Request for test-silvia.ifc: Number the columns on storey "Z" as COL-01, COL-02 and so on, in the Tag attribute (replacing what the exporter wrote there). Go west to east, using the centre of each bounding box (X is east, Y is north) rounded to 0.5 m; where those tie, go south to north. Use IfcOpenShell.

First a look at what the model holds.

```python
import ifcopenshell
import ifcopenshell.util.element
import ifcopenshell.util.placement

model = ifcopenshell.open("test-silvia.ifc")
print(model.schema)
storey = next(s for s in model.by_type("IfcBuildingStorey") if s.Name == "Z")
columns = [e for e in ifcopenshell.util.element.get_decomposition(storey) if e.is_a("IfcColumn")]
for e in sorted(columns, key=lambda e: e.id()):
    origin = ifcopenshell.util.placement.get_local_placement(e.ObjectPlacement)[:3, 3]
    print(e.id(), e.Tag, e.Name, origin.round(2) + 0.0, sep=" | ")
```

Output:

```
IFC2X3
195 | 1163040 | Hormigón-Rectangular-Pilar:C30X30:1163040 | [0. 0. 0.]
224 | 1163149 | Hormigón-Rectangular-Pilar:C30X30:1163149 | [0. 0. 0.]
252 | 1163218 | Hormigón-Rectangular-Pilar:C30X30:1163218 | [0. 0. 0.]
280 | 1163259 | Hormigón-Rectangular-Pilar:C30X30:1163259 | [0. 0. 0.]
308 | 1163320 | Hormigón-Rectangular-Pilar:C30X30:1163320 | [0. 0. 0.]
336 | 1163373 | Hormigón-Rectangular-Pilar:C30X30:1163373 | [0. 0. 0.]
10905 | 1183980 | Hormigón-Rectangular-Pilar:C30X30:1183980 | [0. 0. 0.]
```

```python
import ifcopenshell
import ifcopenshell.geom
import ifcopenshell.util.element
import ifcopenshell.util.shape

model = ifcopenshell.open("test-silvia.ifc")
settings = ifcopenshell.geom.settings()
settings.set("use-world-coords", True)


def centre(element):
    shape = ifcopenshell.geom.create_shape(settings, element)
    return ifcopenshell.util.shape.get_bbox_centroid(shape.geometry)


storey = next(s for s in model.by_type("IfcBuildingStorey") if s.Name == "Z")
columns = [e for e in ifcopenshell.util.element.get_decomposition(storey) if e.is_a("IfcColumn")]

# Insertion points can sit at a corner or the storey origin, so sort by the geometry (in metres).
centres = {e: centre(e) for e in columns}
columns.sort(key=lambda e: (round(centres[e][0] / 0.5), centres[e][1]))

for i, e in enumerate(columns, start=1):
    number = f"COL-{i:02d}"
    e.Tag = number
    print(e.id(), number)

model.write("test-silvia_updated.ifc")
```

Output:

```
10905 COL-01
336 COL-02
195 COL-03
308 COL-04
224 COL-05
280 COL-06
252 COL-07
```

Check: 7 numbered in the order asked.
